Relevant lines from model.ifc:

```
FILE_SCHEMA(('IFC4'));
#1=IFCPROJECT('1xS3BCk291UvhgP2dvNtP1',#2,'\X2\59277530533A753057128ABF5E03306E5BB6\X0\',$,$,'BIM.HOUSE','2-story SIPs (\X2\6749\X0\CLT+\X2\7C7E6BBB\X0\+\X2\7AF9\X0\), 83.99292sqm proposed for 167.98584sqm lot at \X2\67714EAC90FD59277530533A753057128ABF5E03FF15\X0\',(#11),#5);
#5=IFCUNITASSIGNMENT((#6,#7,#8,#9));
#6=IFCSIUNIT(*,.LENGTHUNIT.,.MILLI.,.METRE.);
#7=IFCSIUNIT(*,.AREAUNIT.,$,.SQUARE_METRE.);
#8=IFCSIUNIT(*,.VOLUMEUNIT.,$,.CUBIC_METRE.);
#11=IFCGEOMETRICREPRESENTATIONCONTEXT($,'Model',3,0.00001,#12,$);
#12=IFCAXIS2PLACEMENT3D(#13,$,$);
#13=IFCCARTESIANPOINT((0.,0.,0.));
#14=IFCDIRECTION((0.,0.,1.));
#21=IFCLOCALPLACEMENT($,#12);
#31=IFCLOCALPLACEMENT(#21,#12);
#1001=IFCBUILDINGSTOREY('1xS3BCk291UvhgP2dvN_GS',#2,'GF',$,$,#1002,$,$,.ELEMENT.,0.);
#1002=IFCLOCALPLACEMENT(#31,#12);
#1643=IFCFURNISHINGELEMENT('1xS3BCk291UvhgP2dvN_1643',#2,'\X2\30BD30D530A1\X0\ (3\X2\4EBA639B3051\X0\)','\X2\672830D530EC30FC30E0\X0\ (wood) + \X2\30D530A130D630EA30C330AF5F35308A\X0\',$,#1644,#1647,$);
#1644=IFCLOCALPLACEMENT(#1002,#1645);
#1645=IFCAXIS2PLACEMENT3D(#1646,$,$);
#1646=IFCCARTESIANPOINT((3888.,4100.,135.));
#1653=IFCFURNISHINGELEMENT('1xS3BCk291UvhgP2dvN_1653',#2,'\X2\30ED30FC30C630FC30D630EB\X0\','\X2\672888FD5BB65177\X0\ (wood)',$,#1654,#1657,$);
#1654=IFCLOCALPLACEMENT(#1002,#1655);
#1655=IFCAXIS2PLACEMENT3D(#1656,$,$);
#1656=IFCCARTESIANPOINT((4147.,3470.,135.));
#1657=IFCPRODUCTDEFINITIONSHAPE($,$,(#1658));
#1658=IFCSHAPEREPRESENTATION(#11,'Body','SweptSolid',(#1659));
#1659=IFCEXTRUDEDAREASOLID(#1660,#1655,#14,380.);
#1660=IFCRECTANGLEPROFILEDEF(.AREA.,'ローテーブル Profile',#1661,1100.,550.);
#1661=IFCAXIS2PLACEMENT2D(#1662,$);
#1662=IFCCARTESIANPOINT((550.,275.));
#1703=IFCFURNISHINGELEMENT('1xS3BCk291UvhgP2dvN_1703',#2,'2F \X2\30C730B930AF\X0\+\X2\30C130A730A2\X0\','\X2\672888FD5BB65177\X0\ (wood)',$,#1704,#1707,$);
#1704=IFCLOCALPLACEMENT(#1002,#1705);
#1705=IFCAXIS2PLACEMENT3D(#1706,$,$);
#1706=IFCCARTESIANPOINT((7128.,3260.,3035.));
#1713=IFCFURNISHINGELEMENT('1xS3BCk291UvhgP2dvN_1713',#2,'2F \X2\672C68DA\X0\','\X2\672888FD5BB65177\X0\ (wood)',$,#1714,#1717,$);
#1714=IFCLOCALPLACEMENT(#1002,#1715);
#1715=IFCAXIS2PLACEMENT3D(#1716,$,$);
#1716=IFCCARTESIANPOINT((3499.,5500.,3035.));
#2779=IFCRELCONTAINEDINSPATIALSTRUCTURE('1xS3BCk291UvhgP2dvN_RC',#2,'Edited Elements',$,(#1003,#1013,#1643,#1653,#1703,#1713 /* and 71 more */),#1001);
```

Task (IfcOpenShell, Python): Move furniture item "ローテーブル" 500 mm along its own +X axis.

```python
import ifcopenshell
import ifcopenshell.api.geometry
import ifcopenshell.util.placement

model = ifcopenshell.open("model.ifc")

item = model.by_id(1653)
matrix = ifcopenshell.util.placement.get_local_placement(item.ObjectPlacement)
matrix[:3, 3] += matrix[:3, 0] * 500.0
ifcopenshell.api.geometry.edit_object_placement(model, product=item, matrix=matrix, is_si=False)

print(ifcopenshell.util.placement.get_local_placement(item.ObjectPlacement).round(3) + 0.0)

model.write("model-out.ifc")
```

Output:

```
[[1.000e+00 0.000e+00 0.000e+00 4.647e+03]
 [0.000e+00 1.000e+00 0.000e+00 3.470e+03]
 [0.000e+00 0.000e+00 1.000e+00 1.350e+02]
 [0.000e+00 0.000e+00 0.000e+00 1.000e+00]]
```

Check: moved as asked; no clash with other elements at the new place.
